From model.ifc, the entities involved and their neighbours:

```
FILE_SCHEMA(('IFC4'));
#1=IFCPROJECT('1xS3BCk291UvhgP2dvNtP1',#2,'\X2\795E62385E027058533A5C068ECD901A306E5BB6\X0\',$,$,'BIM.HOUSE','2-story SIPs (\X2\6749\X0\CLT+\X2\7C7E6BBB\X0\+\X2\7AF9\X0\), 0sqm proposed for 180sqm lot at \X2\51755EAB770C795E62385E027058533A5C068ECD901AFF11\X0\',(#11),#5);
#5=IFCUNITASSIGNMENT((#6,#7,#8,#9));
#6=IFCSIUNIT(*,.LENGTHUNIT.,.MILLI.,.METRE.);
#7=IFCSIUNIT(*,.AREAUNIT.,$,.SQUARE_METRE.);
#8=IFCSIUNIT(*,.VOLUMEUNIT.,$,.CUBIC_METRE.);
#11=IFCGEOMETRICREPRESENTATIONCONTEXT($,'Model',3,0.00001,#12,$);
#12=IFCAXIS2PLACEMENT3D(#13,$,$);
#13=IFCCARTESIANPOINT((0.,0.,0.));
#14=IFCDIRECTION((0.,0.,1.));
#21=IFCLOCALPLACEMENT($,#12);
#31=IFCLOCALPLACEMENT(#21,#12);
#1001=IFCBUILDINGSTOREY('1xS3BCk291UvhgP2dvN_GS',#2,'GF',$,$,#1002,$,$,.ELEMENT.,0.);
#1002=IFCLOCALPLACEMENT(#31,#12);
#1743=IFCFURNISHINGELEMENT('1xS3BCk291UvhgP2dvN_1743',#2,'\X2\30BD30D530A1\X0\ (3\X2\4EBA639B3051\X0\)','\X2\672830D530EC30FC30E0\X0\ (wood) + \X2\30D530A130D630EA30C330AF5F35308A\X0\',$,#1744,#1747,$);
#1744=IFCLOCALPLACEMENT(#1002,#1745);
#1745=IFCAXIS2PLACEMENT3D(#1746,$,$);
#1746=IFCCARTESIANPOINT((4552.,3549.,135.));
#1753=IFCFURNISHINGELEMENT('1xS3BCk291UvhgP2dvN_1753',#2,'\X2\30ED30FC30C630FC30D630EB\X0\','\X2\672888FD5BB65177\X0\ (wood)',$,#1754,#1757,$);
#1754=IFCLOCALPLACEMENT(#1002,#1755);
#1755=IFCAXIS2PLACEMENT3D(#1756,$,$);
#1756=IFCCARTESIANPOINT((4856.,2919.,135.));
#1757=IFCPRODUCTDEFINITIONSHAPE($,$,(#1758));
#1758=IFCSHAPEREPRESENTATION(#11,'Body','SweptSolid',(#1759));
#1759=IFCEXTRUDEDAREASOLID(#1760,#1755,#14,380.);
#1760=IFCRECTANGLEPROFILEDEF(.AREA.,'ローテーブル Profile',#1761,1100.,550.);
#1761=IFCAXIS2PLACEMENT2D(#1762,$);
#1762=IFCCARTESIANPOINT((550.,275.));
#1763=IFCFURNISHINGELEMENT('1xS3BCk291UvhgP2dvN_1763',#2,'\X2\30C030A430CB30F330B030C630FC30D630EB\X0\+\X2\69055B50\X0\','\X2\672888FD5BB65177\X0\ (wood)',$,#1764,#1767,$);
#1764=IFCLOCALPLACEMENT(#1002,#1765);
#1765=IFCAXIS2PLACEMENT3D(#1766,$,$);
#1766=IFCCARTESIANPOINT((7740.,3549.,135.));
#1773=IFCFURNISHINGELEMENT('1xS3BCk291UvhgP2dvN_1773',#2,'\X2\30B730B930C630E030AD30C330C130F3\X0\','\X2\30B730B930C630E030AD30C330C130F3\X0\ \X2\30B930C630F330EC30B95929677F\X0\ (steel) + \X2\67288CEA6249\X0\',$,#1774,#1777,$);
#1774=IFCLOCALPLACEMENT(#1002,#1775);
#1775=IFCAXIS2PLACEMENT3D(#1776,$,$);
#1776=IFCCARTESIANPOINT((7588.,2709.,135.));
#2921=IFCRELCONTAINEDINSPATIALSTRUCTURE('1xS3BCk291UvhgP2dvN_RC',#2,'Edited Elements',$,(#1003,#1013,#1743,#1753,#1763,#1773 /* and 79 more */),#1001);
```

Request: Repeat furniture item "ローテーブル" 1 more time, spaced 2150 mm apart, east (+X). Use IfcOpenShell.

```python
import numpy as np
import ifcopenshell
import ifcopenshell.api.geometry
import ifcopenshell.api.root
import ifcopenshell.util.element
import ifcopenshell.util.placement
import ifcopenshell.util.unit

model = ifcopenshell.open("model.ifc")
unit_scale = ifcopenshell.util.unit.calculate_unit_scale(model)


def reuse_history(source, copy):
    """copy_class also copies each property set's owner history, people and application; keep the originals."""
    for rel in copy.IsDefinedBy:
        if rel.is_a("IfcRelDefinesByProperties") and (history := rel.RelatingPropertyDefinition.OwnerHistory):
            rel.RelatingPropertyDefinition.OwnerHistory = source.OwnerHistory
            ifcopenshell.util.element.remove_deep2(model, history)


source = model.by_guid("1xS3BCk291UvhgP2dvN_1753")
base = ifcopenshell.util.placement.get_local_placement(source.ObjectPlacement)
step = np.array([1.0, 0.0, 0.0]) * 2.15 / unit_scale

for i in range(1, 2):
    copy = ifcopenshell.api.root.copy_class(model, product=source)
    copy.Representation = ifcopenshell.util.element.copy_deep(
        model, source.Representation, exclude=["IfcGeometricRepresentationContext", "IfcRepresentationMap"]
    )
    reuse_history(source, copy)
    matrix = base.copy()
    matrix[:3, 3] += i * step
    print("added at", matrix[:3, 3].round(3) + 0.0)
    ifcopenshell.api.geometry.edit_object_placement(model, product=copy, matrix=matrix, is_si=False)

model.write("model-out.ifc")
```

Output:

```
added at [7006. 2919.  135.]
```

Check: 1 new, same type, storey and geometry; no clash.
